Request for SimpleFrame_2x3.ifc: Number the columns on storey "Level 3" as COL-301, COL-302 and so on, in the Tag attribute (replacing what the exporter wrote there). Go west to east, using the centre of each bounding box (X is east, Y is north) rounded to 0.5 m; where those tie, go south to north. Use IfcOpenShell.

First a look at what the model holds.

```python
import ifcopenshell
import ifcopenshell.util.element
import ifcopenshell.util.placement

model = ifcopenshell.open("SimpleFrame_2x3.ifc")
print(model.schema)
storey = next(s for s in model.by_type("IfcBuildingStorey") if s.Name == "Level 3")
columns = [e for e in ifcopenshell.util.element.get_decomposition(storey) if e.is_a("IfcColumn")]
for e in sorted(columns, key=lambda e: e.id()):
    origin = ifcopenshell.util.placement.get_local_placement(e.ObjectPlacement)[:3, 3]
    print(e.id(), e.Tag, e.Name, origin.round(2) + 0.0, sep=" | ")
```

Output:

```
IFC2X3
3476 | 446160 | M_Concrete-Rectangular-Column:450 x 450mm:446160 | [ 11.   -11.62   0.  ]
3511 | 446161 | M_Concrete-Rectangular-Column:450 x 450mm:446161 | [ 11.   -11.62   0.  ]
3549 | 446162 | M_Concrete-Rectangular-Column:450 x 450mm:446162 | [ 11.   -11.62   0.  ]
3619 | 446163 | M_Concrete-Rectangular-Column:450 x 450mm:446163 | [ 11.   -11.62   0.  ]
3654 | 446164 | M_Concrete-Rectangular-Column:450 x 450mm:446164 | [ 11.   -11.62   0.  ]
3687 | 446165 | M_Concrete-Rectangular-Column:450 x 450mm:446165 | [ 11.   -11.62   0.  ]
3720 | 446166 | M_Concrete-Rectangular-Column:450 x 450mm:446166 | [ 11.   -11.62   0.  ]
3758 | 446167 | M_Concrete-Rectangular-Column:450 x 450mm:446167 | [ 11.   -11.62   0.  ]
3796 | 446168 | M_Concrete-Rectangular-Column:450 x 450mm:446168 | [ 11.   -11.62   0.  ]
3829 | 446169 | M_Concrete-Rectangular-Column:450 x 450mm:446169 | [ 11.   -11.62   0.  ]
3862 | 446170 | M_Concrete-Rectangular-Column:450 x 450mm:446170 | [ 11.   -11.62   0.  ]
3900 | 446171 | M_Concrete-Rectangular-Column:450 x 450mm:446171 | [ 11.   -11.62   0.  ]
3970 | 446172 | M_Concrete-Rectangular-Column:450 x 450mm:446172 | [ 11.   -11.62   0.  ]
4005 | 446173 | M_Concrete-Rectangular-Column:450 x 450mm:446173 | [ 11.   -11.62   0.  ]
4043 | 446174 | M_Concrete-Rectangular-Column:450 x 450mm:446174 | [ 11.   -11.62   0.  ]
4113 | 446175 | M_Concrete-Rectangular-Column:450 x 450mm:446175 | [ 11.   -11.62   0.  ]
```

```python
import ifcopenshell
import ifcopenshell.geom
import ifcopenshell.util.element
import ifcopenshell.util.shape

model = ifcopenshell.open("SimpleFrame_2x3.ifc")
settings = ifcopenshell.geom.settings()
settings.set("use-world-coords", True)


def centre(element):
    shape = ifcopenshell.geom.create_shape(settings, element)
    return ifcopenshell.util.shape.get_bbox_centroid(shape.geometry)


storey = next(s for s in model.by_type("IfcBuildingStorey") if s.Name == "Level 3")
columns = [e for e in ifcopenshell.util.element.get_decomposition(storey) if e.is_a("IfcColumn")]

# Insertion points can sit at a corner or the storey origin, so sort by the geometry (in metres).
centres = {e: centre(e) for e in columns}
columns.sort(key=lambda e: (round(centres[e][0] / 0.5), centres[e][1]))

for i, e in enumerate(columns, start=1):
    number = f"COL-3{i:02d}"
    e.Tag = number
    print(e.id(), number)

model.write("SimpleFrame_2x3_v2.ifc")
```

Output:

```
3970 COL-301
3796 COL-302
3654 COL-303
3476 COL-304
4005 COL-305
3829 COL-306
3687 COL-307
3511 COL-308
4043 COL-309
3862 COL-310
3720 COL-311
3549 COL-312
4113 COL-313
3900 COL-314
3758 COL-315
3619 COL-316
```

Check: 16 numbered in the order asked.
